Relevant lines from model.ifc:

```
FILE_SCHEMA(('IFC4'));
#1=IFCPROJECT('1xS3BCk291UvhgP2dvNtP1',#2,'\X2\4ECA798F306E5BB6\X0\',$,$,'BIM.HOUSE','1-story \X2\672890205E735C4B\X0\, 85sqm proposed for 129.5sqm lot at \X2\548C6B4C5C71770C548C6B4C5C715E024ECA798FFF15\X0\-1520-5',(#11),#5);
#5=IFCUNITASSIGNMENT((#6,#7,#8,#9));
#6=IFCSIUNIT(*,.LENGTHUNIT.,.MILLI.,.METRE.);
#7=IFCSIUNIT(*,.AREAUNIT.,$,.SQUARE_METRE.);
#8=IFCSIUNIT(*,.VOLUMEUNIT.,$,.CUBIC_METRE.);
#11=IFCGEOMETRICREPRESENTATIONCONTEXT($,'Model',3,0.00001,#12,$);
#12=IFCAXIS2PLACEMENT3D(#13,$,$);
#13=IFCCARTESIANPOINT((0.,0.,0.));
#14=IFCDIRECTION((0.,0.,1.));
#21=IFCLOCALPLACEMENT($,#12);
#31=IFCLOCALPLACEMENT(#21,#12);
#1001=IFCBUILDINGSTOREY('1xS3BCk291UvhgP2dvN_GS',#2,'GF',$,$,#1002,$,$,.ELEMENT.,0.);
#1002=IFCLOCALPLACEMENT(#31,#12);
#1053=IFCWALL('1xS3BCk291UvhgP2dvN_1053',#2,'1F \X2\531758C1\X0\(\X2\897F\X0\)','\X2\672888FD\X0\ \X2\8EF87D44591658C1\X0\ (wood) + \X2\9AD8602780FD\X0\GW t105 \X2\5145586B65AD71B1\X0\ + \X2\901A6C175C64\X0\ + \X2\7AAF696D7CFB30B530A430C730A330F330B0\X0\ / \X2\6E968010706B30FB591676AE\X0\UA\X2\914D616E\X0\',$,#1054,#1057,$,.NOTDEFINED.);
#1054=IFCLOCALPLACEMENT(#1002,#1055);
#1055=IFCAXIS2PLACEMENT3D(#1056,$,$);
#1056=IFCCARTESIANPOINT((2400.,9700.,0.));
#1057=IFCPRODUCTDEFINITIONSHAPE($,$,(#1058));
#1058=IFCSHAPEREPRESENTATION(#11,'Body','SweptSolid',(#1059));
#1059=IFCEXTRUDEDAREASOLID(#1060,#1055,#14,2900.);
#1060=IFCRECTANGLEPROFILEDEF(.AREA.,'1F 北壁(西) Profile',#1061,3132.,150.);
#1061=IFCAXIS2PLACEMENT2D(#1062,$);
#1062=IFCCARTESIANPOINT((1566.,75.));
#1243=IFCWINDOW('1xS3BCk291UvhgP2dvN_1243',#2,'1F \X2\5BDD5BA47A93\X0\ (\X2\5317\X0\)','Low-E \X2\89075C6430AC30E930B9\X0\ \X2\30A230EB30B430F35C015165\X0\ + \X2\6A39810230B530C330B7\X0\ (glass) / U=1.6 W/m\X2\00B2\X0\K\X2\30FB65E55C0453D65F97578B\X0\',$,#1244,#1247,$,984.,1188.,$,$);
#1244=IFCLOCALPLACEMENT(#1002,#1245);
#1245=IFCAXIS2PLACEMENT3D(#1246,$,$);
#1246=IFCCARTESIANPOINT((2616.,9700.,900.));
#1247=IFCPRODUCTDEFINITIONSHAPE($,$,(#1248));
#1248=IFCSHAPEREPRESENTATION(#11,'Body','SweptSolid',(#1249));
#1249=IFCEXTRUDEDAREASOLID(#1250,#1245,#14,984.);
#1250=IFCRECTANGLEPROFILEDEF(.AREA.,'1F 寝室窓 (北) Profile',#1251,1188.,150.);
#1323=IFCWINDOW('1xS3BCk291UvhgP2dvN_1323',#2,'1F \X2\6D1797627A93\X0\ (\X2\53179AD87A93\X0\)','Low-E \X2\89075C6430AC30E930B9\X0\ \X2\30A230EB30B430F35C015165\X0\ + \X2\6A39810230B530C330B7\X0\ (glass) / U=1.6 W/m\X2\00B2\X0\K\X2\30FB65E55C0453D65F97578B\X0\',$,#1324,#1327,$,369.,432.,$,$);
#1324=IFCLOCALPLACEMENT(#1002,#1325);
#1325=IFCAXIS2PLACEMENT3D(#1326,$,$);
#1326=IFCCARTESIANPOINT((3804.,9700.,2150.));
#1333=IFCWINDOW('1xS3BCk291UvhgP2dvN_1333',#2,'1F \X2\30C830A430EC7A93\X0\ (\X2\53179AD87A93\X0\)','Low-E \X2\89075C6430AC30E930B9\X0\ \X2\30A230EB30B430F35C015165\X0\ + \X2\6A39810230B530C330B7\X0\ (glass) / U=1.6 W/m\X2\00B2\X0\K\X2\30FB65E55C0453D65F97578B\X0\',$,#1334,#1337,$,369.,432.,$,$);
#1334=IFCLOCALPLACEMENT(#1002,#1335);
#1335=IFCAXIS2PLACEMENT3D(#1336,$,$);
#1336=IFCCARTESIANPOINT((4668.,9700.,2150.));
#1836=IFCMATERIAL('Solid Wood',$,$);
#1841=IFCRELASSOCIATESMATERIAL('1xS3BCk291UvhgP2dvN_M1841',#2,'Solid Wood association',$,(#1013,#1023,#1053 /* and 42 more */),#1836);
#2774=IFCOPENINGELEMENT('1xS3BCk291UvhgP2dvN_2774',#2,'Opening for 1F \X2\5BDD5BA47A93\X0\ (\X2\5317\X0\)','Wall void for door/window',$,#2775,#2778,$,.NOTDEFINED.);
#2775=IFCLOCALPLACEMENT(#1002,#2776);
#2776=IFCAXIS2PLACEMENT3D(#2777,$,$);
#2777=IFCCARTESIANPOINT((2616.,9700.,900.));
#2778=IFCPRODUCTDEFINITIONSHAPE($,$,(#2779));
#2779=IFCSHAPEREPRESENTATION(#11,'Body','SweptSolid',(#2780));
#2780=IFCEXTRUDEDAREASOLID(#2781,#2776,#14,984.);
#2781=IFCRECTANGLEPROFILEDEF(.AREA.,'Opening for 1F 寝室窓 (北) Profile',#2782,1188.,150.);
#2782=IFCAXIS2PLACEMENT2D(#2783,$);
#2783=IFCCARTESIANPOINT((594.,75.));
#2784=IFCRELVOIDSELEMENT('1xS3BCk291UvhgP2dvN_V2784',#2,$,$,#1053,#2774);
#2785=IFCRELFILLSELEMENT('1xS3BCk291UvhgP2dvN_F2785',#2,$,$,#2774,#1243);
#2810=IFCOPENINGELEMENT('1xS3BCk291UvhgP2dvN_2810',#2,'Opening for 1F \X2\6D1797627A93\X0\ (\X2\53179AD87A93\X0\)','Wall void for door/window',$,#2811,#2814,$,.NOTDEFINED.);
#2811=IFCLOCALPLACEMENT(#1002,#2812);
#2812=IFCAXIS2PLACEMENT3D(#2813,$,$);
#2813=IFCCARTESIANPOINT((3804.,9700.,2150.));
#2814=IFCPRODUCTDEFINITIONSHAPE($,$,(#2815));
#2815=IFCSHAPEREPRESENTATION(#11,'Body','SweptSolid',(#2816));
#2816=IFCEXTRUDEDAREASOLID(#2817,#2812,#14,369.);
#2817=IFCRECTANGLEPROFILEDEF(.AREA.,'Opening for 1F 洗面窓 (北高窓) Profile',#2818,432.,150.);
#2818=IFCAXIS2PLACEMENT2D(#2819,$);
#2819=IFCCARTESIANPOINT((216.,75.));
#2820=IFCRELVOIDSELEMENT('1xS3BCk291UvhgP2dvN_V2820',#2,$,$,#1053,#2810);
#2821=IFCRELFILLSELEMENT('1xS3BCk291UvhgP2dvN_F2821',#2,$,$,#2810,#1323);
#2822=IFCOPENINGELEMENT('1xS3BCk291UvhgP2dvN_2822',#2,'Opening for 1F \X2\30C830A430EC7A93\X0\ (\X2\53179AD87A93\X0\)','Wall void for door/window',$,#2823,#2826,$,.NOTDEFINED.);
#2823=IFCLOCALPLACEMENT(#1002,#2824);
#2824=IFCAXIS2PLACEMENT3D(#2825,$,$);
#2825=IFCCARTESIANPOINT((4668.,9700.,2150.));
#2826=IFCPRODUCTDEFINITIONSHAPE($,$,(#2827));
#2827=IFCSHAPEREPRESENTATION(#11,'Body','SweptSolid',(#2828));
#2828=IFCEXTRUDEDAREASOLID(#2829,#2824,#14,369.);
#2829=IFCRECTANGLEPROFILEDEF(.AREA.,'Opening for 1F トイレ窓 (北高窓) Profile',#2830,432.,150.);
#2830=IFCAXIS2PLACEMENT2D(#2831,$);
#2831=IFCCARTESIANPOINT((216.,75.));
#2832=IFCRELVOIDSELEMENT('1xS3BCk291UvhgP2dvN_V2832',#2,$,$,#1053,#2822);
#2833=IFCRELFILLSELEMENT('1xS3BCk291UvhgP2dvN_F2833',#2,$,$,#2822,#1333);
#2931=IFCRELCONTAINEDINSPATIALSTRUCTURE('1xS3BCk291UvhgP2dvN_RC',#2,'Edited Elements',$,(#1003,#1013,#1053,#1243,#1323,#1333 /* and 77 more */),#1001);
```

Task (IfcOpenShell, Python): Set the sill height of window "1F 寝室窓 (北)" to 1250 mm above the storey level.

```python
import numpy as np
import ifcopenshell
import ifcopenshell.api.geometry
import ifcopenshell.geom
import ifcopenshell.util.element
import ifcopenshell.util.placement
import ifcopenshell.util.shape
import ifcopenshell.util.unit

model = ifcopenshell.open("model.ifc")
unit_scale = ifcopenshell.util.unit.calculate_unit_scale(model)

window = model.by_id(1243)
opening = window.FillsVoids[0].RelatingOpeningElement
storey = ifcopenshell.util.element.get_container(window, ifc_class="IfcBuildingStorey")
level = ifcopenshell.util.placement.get_local_placement(storey.ObjectPlacement)[2, 3]

# The opening's origin need not be at the sill, so measure its lowest point.
shape = ifcopenshell.geom.create_shape(ifcopenshell.geom.settings(), opening)
bottom = ifcopenshell.util.shape.get_shape_bottom_elevation(shape, shape.geometry) / unit_scale
dz = level + 1.25 / unit_scale - bottom

shift = np.array([0.0, 0.0, dz])
# The window is not placed relative to its opening, so move both.
for product in (opening, window):
    matrix = ifcopenshell.util.placement.get_local_placement(product.ObjectPlacement)
    matrix[:3, 3] += shift
    ifcopenshell.api.geometry.edit_object_placement(model, product=product, matrix=matrix, is_si=False)

print(f"moved by {dz * unit_scale:+.3f} m")

model.write("model_rev.ifc")
```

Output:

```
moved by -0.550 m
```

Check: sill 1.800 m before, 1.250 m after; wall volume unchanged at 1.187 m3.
